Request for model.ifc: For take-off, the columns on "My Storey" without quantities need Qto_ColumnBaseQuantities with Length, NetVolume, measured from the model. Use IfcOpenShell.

First a look at what the model holds.

```python
import ifcopenshell
import ifcopenshell.util.element
import ifcopenshell.util.unit

model = ifcopenshell.open("model.ifc")
print(model.schema)
for unit_type in ("LENGTHUNIT", "AREAUNIT", "VOLUMEUNIT"):
    print(unit_type, ifcopenshell.util.unit.calculate_unit_scale(model, unit_type))
storey = next(s for s in model.by_type("IfcBuildingStorey") if s.Name == "My Storey")
columns = [e for e in ifcopenshell.util.element.get_decomposition(storey) if e.is_a("IfcColumn")]
for e in sorted(columns, key=lambda e: e.id()):
    print(e.id(), e.is_a(), e.Name, list(ifcopenshell.util.element.get_psets(e, qtos_only=True)), sep=" | ")
```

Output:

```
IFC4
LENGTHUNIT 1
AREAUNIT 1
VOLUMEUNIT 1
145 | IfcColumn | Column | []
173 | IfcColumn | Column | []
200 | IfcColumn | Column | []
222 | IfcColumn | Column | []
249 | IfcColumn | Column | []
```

```python
import ifcopenshell
import ifcopenshell.api.pset
import ifcopenshell.geom
import ifcopenshell.util.element
import ifcopenshell.util.shape
import ifcopenshell.util.unit

model = ifcopenshell.open("model.ifc")
unit_scale = ifcopenshell.util.unit.calculate_unit_scale(model)
volume_scale = ifcopenshell.util.unit.calculate_unit_scale(model, "VOLUMEUNIT")
settings = ifcopenshell.geom.settings()

storey = next(s for s in model.by_type("IfcBuildingStorey") if s.Name == "My Storey")
columns = [e for e in ifcopenshell.util.element.get_decomposition(storey) if e.is_a("IfcColumn")]

for e in sorted(columns, key=lambda e: e.id()):
    if ifcopenshell.util.element.get_psets(e, qtos_only=True, should_inherit=False):
        continue
    # Geometry comes back in metres, in the element's own axes.
    shape = ifcopenshell.geom.create_shape(settings, e)
    values = {
        "Length": ifcopenshell.util.shape.get_z(shape.geometry) / unit_scale,
        "NetVolume": ifcopenshell.util.shape.get_volume(shape.geometry) / volume_scale,
    }
    qto = ifcopenshell.api.pset.add_qto(model, product=e, name="Qto_ColumnBaseQuantities")
    ifcopenshell.api.pset.edit_qto(model, qto=qto, properties=values)
    print(e.id(), {k: round(v, 3) for k, v in values.items()})

model.write("model-out.ifc")
```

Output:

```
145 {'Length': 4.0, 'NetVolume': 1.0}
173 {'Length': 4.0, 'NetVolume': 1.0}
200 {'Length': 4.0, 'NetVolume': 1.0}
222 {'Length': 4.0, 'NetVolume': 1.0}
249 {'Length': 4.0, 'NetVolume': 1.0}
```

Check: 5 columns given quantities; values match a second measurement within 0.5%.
